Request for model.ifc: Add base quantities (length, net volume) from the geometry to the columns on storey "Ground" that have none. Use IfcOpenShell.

First a look at what the model holds.

```python
import ifcopenshell
import ifcopenshell.util.element
import ifcopenshell.util.unit

model = ifcopenshell.open("model.ifc")
print(model.schema)
for unit_type in ("LENGTHUNIT", "AREAUNIT", "VOLUMEUNIT"):
    print(unit_type, ifcopenshell.util.unit.calculate_unit_scale(model, unit_type))
storey = next(s for s in model.by_type("IfcBuildingStorey") if s.Name == "Ground")
columns = [e for e in ifcopenshell.util.element.get_decomposition(storey) if e.is_a("IfcColumn")]
for e in sorted(columns, key=lambda e: e.id()):
    print(e.id(), e.is_a(), e.Name, list(ifcopenshell.util.element.get_psets(e, qtos_only=True)), sep=" | ")
```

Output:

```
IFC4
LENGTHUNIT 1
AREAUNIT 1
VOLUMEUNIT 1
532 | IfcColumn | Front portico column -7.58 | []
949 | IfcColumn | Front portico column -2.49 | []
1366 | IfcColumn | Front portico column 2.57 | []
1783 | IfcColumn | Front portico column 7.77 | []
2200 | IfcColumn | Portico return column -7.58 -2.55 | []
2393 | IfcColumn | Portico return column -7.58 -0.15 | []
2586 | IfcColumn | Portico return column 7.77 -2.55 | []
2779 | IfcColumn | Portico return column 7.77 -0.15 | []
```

```python
import ifcopenshell
import ifcopenshell.api.pset
import ifcopenshell.geom
import ifcopenshell.util.element
import ifcopenshell.util.shape
import ifcopenshell.util.unit

model = ifcopenshell.open("model.ifc")
unit_scale = ifcopenshell.util.unit.calculate_unit_scale(model)
volume_scale = ifcopenshell.util.unit.calculate_unit_scale(model, "VOLUMEUNIT")
settings = ifcopenshell.geom.settings()

storey = next(s for s in model.by_type("IfcBuildingStorey") if s.Name == "Ground")
columns = [e for e in ifcopenshell.util.element.get_decomposition(storey) if e.is_a("IfcColumn")]

for e in sorted(columns, key=lambda e: e.id()):
    if ifcopenshell.util.element.get_psets(e, qtos_only=True, should_inherit=False):
        continue
    # Geometry comes back in metres, in the element's own axes.
    shape = ifcopenshell.geom.create_shape(settings, e)
    values = {
        "Length": ifcopenshell.util.shape.get_z(shape.geometry) / unit_scale,
        "NetVolume": ifcopenshell.util.shape.get_volume(shape.geometry) / volume_scale,
    }
    qto = ifcopenshell.api.pset.add_qto(model, product=e, name="Qto_ColumnBaseQuantities")
    ifcopenshell.api.pset.edit_qto(model, qto=qto, properties=values)
    print(e.id(), {k: round(v, 3) for k, v in values.items()})

model.write("model-out.ifc")
```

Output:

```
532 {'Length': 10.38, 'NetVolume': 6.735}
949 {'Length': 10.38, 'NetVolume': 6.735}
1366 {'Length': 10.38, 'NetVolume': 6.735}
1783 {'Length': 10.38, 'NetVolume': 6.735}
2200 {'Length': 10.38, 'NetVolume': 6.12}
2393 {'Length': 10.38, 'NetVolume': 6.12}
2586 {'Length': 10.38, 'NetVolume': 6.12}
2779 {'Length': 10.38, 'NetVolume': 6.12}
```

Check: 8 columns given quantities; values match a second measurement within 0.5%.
